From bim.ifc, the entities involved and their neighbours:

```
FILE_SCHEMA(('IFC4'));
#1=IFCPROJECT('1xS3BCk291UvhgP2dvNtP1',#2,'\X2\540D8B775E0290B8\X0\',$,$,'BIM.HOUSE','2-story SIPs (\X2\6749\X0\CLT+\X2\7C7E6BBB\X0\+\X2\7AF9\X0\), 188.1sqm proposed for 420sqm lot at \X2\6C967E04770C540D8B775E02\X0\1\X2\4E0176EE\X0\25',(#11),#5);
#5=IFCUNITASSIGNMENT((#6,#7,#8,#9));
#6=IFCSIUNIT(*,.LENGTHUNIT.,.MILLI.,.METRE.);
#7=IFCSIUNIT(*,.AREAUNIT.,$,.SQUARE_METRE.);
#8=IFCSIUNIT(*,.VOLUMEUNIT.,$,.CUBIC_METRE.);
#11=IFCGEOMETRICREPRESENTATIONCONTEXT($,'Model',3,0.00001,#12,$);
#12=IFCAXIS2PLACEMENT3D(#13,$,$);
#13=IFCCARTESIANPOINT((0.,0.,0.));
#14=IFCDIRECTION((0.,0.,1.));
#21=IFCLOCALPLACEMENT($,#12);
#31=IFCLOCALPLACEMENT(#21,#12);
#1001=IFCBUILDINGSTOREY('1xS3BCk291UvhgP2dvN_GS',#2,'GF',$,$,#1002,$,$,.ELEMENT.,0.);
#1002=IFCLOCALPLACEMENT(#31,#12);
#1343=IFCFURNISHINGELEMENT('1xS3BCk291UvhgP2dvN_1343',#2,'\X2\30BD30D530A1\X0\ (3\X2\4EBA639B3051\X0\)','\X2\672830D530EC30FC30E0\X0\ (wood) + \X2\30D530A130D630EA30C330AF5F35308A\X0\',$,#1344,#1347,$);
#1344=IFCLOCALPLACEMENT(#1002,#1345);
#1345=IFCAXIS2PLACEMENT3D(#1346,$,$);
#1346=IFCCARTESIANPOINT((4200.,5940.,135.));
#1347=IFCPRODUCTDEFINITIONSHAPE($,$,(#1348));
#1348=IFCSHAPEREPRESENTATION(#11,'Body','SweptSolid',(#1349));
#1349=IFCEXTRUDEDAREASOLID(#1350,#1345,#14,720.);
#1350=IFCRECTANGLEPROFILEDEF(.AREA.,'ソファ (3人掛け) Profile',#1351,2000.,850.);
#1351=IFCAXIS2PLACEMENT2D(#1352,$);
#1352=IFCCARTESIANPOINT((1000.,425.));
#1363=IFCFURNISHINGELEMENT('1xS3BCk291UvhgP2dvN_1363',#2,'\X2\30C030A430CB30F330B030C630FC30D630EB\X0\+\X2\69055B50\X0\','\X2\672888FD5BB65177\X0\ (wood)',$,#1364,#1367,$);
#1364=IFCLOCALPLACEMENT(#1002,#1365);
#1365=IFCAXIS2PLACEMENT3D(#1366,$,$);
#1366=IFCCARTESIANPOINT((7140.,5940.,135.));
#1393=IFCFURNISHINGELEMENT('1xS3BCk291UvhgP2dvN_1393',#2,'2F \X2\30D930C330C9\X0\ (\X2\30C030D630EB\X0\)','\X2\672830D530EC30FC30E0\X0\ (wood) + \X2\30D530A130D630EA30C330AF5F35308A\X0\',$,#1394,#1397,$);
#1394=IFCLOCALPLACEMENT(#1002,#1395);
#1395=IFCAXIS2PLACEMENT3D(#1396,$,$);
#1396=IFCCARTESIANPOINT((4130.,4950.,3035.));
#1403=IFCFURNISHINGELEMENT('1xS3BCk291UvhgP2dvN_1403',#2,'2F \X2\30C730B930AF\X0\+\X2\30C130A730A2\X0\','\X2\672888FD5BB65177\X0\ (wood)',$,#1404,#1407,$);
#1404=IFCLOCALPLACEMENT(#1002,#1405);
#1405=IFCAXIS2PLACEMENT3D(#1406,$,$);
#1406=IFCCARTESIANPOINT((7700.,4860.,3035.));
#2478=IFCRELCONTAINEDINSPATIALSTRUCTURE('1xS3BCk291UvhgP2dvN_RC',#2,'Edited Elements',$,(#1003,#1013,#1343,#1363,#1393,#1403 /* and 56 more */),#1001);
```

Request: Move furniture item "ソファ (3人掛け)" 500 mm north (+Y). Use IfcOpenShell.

```python
import ifcopenshell
import ifcopenshell.api.geometry
import ifcopenshell.util.placement
import ifcopenshell.util.unit

model = ifcopenshell.open("bim.ifc")
unit_scale = ifcopenshell.util.unit.calculate_unit_scale(model)

item = model.by_id(1343)
matrix = ifcopenshell.util.placement.get_local_placement(item.ObjectPlacement)
matrix[1, 3] += 0.5 / unit_scale
ifcopenshell.api.geometry.edit_object_placement(model, product=item, matrix=matrix, is_si=False)

print(ifcopenshell.util.placement.get_local_placement(item.ObjectPlacement).round(3) + 0.0)

model.write("bim_edited.ifc")
```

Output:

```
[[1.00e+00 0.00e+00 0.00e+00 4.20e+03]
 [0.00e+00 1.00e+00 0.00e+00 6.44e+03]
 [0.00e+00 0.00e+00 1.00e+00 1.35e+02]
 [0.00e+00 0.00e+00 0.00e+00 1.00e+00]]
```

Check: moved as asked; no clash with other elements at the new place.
